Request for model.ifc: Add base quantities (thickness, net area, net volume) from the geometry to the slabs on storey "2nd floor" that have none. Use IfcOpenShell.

First a look at what the model holds.

```python
import ifcopenshell
import ifcopenshell.util.element
import ifcopenshell.util.unit

model = ifcopenshell.open("model.ifc")
print(model.schema)
for unit_type in ("LENGTHUNIT", "AREAUNIT", "VOLUMEUNIT"):
    print(unit_type, ifcopenshell.util.unit.calculate_unit_scale(model, unit_type))
storey = next(s for s in model.by_type("IfcBuildingStorey") if s.Name == "2nd floor")
slabs = [e for e in ifcopenshell.util.element.get_decomposition(storey) if e.is_a("IfcSlab")]
for e in sorted(slabs, key=lambda e: e.id()):
    print(e.id(), e.is_a(), e.Name, list(ifcopenshell.util.element.get_psets(e, qtos_only=True)), sep=" | ")
```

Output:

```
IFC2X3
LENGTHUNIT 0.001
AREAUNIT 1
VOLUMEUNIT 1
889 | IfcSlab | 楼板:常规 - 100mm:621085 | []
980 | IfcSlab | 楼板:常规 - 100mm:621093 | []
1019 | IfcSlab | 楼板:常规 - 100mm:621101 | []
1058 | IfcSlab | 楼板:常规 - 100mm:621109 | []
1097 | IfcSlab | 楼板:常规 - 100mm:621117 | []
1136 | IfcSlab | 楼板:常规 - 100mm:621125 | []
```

```python
import ifcopenshell
import ifcopenshell.api.pset
import ifcopenshell.geom
import ifcopenshell.util.element
import ifcopenshell.util.shape
import ifcopenshell.util.unit

model = ifcopenshell.open("model.ifc")
unit_scale = ifcopenshell.util.unit.calculate_unit_scale(model)
area_scale = ifcopenshell.util.unit.calculate_unit_scale(model, "AREAUNIT")
volume_scale = ifcopenshell.util.unit.calculate_unit_scale(model, "VOLUMEUNIT")
settings = ifcopenshell.geom.settings()

storey = next(s for s in model.by_type("IfcBuildingStorey") if s.Name == "2nd floor")
slabs = [e for e in ifcopenshell.util.element.get_decomposition(storey) if e.is_a("IfcSlab")]

for e in sorted(slabs, key=lambda e: e.id()):
    if ifcopenshell.util.element.get_psets(e, qtos_only=True, should_inherit=False):
        continue
    # Geometry comes back in metres, in the element's own axes.
    shape = ifcopenshell.geom.create_shape(settings, e)
    values = {
        "Width": ifcopenshell.util.shape.get_z(shape.geometry) / unit_scale,
        "NetArea": ifcopenshell.util.shape.get_footprint_area(shape.geometry) / area_scale,
        "NetVolume": ifcopenshell.util.shape.get_volume(shape.geometry) / volume_scale,
    }
    qto = ifcopenshell.api.pset.add_qto(model, product=e, name="BaseQuantities")
    ifcopenshell.api.pset.edit_qto(model, qto=qto, properties=values)
    print(e.id(), {k: round(v, 3) for k, v in values.items()})

model.write("model_v2.ifc")
```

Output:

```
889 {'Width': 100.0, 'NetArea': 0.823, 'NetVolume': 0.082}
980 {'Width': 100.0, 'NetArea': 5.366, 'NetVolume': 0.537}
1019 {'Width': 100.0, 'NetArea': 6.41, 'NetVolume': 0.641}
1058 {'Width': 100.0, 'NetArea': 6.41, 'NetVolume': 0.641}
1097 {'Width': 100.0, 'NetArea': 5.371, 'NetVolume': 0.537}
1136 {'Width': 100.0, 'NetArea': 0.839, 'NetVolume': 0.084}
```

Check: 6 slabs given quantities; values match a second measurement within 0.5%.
